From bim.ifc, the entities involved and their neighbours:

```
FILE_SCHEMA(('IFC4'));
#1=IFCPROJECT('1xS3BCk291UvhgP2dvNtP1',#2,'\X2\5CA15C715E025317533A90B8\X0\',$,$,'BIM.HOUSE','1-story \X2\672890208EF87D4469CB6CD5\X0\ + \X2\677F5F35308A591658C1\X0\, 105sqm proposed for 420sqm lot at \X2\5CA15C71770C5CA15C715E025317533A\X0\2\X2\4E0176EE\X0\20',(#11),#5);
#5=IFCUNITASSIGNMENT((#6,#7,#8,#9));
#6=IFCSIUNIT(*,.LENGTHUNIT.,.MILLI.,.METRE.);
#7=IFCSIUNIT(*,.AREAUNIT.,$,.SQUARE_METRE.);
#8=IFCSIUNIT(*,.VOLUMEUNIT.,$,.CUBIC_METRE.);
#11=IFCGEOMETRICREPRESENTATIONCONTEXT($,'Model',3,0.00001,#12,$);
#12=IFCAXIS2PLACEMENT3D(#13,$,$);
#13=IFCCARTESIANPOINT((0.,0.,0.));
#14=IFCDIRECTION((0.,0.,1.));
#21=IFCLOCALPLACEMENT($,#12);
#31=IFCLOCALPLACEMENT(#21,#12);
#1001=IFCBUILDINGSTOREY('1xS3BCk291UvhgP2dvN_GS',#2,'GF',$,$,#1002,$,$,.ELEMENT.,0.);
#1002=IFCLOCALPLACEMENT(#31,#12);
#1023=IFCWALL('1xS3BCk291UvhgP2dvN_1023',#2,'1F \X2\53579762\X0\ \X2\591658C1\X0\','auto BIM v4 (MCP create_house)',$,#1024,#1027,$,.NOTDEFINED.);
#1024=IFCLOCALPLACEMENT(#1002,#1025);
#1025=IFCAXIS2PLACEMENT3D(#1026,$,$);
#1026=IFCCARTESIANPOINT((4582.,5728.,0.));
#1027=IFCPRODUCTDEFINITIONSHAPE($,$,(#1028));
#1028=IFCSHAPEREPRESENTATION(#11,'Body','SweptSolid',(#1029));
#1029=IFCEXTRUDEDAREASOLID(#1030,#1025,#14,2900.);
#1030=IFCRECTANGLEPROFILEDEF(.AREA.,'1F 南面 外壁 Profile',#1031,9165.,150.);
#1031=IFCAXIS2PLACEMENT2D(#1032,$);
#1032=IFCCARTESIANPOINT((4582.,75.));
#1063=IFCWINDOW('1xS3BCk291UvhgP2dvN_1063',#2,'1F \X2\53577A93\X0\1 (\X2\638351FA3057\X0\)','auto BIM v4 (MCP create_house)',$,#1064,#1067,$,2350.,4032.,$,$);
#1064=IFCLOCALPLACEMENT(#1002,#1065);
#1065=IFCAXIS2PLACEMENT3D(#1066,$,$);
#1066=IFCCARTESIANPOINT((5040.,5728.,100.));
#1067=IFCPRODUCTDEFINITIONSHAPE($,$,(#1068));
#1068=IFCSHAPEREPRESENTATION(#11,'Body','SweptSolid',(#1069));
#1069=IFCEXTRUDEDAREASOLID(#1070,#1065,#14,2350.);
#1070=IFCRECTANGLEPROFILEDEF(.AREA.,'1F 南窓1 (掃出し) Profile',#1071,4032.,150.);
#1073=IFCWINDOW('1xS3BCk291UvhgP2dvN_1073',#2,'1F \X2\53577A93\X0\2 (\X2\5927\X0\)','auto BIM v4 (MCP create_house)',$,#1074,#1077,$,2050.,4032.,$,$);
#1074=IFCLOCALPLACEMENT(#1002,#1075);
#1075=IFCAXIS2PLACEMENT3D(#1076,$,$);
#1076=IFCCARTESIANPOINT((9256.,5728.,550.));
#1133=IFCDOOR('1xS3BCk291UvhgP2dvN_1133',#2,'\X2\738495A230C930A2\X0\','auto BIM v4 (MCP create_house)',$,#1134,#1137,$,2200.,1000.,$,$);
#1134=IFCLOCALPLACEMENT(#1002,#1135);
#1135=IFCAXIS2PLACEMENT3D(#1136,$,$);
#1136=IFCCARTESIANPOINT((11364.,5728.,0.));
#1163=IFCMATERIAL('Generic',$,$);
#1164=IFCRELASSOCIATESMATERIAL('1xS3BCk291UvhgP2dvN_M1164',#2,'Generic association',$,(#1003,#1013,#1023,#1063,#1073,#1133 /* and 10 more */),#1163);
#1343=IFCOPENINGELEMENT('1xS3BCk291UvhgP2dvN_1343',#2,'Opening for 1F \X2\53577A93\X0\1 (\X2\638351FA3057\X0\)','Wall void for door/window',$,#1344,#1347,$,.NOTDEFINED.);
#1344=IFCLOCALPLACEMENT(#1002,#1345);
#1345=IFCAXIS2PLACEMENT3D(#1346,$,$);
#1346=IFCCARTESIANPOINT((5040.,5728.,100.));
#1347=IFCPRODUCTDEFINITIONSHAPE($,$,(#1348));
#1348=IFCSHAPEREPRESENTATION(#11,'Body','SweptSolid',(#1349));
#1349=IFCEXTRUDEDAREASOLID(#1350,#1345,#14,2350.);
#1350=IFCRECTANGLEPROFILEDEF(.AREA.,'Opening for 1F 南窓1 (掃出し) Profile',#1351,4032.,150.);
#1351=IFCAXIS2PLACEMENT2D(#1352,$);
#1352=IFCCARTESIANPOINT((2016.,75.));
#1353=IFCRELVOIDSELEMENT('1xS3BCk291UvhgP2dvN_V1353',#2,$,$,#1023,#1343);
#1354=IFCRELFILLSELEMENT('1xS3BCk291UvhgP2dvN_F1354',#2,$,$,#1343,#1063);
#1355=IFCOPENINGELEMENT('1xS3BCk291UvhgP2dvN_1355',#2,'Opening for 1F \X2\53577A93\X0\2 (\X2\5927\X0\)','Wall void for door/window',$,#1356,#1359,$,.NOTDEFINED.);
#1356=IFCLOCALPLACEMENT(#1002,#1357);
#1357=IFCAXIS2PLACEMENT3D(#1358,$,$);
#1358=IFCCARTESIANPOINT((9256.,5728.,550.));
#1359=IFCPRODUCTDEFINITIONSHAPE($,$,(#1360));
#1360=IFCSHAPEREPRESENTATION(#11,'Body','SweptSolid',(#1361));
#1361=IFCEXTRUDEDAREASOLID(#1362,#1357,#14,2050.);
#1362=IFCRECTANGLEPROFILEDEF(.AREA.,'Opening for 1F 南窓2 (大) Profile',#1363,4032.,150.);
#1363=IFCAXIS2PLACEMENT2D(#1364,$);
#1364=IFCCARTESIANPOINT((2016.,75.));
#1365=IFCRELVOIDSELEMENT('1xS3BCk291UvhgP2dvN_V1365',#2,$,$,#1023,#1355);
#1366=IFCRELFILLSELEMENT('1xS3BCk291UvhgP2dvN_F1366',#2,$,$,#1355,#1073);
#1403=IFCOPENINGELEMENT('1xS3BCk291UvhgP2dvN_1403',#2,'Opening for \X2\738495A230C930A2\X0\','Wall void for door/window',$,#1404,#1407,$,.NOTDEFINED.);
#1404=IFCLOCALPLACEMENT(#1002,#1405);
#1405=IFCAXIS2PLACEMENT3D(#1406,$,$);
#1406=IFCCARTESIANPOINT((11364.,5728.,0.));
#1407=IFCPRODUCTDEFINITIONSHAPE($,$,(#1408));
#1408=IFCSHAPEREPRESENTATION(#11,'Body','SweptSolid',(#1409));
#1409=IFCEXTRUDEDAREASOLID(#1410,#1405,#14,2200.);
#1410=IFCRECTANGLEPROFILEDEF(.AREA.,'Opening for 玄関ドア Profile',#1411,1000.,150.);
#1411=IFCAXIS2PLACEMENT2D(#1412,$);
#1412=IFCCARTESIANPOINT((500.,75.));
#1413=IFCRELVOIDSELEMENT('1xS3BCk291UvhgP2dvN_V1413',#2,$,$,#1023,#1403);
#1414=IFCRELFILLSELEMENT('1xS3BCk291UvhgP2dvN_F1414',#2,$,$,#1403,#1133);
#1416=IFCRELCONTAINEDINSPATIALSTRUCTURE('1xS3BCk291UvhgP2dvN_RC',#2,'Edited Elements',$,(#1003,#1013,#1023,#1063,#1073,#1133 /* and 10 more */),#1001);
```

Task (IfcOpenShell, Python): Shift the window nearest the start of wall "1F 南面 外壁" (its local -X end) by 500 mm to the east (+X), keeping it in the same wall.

```python
import ifcopenshell
import ifcopenshell.api.geometry
import ifcopenshell.util.placement
import ifcopenshell.util.unit

model = ifcopenshell.open("bim.ifc")
unit_scale = ifcopenshell.util.unit.calculate_unit_scale(model)

window = model.by_guid("1xS3BCk291UvhgP2dvN_1063")
opening = window.FillsVoids[0].RelatingOpeningElement
wall = opening.VoidsElements[0].RelatingBuildingElement

wall_matrix = ifcopenshell.util.placement.get_local_placement(wall.ObjectPlacement)
shift = wall_matrix[:3, 0] * 0.5 / unit_scale
before = ifcopenshell.util.placement.get_local_placement(window.ObjectPlacement)[:3, 3].copy()

# The window is not placed relative to its opening, so move both.
for product in (opening, window):
    matrix = ifcopenshell.util.placement.get_local_placement(product.ObjectPlacement)
    matrix[:3, 3] += shift
    ifcopenshell.api.geometry.edit_object_placement(model, product=product, matrix=matrix, is_si=False)

after = ifcopenshell.util.placement.get_local_placement(window.ObjectPlacement)[:3, 3]
print("window moved by", (after - before).round(3) + 0.0)

model.write("bim_edited.ifc")
```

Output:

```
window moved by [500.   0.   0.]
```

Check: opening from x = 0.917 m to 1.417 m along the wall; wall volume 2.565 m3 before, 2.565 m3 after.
